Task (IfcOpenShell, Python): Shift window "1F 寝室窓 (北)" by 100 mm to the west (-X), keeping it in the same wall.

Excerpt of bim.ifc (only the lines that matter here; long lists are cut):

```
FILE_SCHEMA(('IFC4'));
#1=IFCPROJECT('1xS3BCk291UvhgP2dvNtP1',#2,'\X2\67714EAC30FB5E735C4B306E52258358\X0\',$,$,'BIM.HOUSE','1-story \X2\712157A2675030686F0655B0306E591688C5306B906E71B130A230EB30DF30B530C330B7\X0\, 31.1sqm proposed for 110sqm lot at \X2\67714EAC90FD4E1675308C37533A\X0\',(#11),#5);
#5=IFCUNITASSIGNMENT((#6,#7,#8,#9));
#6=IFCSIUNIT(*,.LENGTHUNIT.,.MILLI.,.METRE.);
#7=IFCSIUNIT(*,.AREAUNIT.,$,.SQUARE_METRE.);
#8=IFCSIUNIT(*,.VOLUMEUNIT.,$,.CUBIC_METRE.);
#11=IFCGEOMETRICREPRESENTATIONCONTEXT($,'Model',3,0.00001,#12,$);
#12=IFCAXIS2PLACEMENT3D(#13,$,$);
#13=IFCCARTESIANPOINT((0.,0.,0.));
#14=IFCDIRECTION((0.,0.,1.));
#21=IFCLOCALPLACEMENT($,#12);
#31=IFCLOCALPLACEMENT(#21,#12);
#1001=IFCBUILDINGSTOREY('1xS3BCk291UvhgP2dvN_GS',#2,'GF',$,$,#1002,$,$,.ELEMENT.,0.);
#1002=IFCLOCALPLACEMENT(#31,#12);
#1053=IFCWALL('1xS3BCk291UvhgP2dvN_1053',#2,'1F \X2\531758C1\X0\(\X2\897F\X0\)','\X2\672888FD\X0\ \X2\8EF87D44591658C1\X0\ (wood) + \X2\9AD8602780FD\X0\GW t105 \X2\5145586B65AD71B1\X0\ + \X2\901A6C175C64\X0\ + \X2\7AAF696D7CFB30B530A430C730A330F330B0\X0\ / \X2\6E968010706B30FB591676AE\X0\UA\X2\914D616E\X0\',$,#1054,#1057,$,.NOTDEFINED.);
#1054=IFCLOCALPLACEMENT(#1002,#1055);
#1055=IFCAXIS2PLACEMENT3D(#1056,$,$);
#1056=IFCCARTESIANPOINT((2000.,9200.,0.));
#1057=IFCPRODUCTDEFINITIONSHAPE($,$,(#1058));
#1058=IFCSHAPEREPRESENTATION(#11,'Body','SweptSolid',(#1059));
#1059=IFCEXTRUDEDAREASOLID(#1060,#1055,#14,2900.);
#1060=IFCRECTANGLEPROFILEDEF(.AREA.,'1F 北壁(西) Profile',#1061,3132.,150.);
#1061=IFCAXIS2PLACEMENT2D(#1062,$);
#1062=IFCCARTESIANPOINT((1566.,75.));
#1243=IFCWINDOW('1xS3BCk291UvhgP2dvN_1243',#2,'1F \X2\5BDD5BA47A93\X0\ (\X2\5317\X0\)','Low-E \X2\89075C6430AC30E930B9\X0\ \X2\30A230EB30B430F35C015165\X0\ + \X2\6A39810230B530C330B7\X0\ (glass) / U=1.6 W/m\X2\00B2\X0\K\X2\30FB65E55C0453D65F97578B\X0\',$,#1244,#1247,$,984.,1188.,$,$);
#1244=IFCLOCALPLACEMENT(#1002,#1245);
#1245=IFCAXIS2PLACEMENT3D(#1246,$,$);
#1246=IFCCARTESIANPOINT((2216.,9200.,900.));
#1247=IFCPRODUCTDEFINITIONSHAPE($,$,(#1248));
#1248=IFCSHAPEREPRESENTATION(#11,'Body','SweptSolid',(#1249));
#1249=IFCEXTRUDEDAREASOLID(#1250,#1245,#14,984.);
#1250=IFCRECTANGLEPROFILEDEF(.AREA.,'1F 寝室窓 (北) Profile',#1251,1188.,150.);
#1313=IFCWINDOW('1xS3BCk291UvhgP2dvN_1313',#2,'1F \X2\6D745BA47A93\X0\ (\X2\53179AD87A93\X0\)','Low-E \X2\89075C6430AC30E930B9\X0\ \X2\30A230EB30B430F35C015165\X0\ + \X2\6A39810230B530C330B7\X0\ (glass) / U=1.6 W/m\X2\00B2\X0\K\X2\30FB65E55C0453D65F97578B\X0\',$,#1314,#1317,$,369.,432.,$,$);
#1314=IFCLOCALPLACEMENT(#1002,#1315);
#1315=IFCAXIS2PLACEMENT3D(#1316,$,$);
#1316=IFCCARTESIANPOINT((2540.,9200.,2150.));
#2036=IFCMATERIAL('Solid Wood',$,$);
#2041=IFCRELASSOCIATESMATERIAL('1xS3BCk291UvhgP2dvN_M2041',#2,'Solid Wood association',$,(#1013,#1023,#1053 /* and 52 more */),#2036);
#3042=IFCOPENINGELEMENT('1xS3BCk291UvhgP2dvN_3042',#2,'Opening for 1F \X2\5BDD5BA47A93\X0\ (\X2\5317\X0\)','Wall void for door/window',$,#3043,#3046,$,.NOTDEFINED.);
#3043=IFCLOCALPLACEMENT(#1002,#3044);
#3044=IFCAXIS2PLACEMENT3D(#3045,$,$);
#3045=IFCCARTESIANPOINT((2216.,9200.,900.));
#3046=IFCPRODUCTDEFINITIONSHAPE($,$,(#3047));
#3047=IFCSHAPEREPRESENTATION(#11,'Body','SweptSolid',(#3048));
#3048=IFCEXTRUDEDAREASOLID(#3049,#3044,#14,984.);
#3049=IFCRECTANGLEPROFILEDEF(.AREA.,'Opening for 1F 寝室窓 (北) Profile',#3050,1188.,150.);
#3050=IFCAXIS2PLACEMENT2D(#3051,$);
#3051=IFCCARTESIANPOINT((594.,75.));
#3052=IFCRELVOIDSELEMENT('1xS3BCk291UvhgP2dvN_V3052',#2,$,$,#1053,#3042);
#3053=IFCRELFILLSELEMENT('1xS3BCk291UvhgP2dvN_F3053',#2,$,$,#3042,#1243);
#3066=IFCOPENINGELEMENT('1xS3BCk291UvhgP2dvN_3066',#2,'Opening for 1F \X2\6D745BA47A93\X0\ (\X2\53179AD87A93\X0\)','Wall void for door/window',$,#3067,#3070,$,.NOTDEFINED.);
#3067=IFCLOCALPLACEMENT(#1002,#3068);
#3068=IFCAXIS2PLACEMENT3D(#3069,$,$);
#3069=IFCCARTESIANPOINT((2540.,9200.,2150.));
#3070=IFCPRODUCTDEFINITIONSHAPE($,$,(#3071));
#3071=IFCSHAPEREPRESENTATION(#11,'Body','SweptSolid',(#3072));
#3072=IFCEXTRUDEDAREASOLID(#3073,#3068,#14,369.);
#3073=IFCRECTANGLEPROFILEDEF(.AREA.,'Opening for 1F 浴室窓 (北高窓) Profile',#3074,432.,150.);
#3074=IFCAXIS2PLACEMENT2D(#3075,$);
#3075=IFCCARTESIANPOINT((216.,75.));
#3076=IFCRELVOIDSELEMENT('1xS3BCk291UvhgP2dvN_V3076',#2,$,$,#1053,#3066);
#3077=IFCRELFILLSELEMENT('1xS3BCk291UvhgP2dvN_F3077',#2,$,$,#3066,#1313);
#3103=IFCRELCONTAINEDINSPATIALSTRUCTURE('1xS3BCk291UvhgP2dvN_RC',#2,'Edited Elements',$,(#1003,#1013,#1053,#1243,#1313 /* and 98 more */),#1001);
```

```python
import ifcopenshell
import ifcopenshell.api.geometry
import ifcopenshell.util.placement

model = ifcopenshell.open("bim.ifc")

window = model.by_guid("1xS3BCk291UvhgP2dvN_1243")
opening = window.FillsVoids[0].RelatingOpeningElement
wall = opening.VoidsElements[0].RelatingBuildingElement

wall_matrix = ifcopenshell.util.placement.get_local_placement(wall.ObjectPlacement)
shift = wall_matrix[:3, 0] * -100.0
before = ifcopenshell.util.placement.get_local_placement(window.ObjectPlacement)[:3, 3].copy()

# The window is not placed relative to its opening, so move both.
for product in (opening, window):
    matrix = ifcopenshell.util.placement.get_local_placement(product.ObjectPlacement)
    matrix[:3, 3] += shift
    ifcopenshell.api.geometry.edit_object_placement(model, product=product, matrix=matrix, is_si=False)

after = ifcopenshell.util.placement.get_local_placement(window.ObjectPlacement)[:3, 3]
print("window moved by", (after - before).round(3) + 0.0)

model.write("bim_v2.ifc")
```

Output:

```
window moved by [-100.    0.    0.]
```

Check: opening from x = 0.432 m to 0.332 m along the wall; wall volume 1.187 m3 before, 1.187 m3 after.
